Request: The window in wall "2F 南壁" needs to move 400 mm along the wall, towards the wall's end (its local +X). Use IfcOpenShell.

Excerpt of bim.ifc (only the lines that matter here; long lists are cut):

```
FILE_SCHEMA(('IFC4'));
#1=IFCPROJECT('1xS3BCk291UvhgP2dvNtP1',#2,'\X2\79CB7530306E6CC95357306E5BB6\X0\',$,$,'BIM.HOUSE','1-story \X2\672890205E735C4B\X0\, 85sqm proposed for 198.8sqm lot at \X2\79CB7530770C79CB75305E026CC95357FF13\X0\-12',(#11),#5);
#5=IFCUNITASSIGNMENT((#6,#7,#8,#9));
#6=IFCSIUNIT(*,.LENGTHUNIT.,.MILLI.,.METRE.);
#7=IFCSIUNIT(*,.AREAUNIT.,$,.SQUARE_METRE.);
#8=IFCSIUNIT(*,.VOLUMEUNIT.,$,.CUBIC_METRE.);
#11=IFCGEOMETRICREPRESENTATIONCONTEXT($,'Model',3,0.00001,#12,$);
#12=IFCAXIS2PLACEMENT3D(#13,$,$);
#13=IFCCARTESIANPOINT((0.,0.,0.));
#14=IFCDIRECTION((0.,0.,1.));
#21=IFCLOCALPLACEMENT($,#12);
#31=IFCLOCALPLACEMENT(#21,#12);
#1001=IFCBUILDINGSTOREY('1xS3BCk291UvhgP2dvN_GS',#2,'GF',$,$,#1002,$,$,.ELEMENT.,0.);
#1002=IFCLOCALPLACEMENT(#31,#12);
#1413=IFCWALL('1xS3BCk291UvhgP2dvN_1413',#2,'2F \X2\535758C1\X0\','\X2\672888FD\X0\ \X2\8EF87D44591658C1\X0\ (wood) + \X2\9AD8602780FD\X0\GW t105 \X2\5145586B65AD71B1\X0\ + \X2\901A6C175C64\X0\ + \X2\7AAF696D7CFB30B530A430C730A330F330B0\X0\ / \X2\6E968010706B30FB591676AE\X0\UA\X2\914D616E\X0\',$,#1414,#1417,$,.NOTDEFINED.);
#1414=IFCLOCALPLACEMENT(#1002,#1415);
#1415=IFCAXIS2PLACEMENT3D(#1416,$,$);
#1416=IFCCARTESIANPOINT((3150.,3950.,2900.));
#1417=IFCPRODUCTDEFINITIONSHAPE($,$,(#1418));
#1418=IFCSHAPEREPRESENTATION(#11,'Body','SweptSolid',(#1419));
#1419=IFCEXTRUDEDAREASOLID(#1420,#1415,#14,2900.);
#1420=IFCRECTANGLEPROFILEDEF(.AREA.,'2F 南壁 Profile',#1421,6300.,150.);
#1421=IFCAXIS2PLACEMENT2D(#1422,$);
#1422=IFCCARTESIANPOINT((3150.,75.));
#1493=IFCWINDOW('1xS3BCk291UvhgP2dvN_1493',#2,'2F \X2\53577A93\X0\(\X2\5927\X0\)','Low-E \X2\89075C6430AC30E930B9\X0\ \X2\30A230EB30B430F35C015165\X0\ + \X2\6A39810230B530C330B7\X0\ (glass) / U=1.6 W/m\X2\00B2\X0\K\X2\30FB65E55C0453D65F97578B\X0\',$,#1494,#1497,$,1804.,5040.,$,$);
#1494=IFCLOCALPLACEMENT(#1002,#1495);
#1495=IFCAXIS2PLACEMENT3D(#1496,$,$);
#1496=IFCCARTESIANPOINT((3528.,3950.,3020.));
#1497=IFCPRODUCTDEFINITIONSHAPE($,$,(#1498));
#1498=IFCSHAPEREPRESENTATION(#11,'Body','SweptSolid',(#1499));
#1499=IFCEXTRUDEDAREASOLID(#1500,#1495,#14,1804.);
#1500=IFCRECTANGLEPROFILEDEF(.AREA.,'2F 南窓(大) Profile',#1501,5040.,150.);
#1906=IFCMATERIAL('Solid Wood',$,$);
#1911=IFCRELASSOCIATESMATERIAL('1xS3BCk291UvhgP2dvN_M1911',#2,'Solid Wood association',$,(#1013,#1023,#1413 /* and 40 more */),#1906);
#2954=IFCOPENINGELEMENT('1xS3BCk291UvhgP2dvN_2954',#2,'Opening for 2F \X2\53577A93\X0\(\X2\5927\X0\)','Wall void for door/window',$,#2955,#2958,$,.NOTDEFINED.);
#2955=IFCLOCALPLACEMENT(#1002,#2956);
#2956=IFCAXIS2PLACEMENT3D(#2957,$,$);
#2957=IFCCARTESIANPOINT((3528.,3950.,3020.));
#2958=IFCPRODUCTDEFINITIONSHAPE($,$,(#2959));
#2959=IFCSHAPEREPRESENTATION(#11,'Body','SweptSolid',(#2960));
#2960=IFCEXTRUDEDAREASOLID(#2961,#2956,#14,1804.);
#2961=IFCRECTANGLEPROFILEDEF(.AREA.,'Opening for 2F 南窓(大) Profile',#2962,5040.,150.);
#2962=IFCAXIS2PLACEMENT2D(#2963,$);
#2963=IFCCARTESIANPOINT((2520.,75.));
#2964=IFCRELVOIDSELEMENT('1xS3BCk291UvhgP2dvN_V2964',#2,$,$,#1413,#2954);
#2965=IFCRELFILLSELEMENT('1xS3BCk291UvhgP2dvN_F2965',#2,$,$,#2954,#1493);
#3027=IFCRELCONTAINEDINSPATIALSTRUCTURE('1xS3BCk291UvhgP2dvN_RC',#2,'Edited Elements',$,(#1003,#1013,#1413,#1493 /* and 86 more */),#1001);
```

```python
import ifcopenshell
import ifcopenshell.api.geometry
import ifcopenshell.util.placement

model = ifcopenshell.open("bim.ifc")

window = model.by_guid("1xS3BCk291UvhgP2dvN_1493")
opening = window.FillsVoids[0].RelatingOpeningElement
wall = opening.VoidsElements[0].RelatingBuildingElement

wall_matrix = ifcopenshell.util.placement.get_local_placement(wall.ObjectPlacement)
shift = wall_matrix[:3, 0] * 400.0
before = ifcopenshell.util.placement.get_local_placement(window.ObjectPlacement)[:3, 3].copy()

# The window is not placed relative to its opening, so move both.
for product in (opening, window):
    matrix = ifcopenshell.util.placement.get_local_placement(product.ObjectPlacement)
    matrix[:3, 3] += shift
    ifcopenshell.api.geometry.edit_object_placement(model, product=product, matrix=matrix, is_si=False)

after = ifcopenshell.util.placement.get_local_placement(window.ObjectPlacement)[:3, 3]
print("window moved by", (after - before).round(3) + 0.0)

model.write("bim_v2.ifc")
```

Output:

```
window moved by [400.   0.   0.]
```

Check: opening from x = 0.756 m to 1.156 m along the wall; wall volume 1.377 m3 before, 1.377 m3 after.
